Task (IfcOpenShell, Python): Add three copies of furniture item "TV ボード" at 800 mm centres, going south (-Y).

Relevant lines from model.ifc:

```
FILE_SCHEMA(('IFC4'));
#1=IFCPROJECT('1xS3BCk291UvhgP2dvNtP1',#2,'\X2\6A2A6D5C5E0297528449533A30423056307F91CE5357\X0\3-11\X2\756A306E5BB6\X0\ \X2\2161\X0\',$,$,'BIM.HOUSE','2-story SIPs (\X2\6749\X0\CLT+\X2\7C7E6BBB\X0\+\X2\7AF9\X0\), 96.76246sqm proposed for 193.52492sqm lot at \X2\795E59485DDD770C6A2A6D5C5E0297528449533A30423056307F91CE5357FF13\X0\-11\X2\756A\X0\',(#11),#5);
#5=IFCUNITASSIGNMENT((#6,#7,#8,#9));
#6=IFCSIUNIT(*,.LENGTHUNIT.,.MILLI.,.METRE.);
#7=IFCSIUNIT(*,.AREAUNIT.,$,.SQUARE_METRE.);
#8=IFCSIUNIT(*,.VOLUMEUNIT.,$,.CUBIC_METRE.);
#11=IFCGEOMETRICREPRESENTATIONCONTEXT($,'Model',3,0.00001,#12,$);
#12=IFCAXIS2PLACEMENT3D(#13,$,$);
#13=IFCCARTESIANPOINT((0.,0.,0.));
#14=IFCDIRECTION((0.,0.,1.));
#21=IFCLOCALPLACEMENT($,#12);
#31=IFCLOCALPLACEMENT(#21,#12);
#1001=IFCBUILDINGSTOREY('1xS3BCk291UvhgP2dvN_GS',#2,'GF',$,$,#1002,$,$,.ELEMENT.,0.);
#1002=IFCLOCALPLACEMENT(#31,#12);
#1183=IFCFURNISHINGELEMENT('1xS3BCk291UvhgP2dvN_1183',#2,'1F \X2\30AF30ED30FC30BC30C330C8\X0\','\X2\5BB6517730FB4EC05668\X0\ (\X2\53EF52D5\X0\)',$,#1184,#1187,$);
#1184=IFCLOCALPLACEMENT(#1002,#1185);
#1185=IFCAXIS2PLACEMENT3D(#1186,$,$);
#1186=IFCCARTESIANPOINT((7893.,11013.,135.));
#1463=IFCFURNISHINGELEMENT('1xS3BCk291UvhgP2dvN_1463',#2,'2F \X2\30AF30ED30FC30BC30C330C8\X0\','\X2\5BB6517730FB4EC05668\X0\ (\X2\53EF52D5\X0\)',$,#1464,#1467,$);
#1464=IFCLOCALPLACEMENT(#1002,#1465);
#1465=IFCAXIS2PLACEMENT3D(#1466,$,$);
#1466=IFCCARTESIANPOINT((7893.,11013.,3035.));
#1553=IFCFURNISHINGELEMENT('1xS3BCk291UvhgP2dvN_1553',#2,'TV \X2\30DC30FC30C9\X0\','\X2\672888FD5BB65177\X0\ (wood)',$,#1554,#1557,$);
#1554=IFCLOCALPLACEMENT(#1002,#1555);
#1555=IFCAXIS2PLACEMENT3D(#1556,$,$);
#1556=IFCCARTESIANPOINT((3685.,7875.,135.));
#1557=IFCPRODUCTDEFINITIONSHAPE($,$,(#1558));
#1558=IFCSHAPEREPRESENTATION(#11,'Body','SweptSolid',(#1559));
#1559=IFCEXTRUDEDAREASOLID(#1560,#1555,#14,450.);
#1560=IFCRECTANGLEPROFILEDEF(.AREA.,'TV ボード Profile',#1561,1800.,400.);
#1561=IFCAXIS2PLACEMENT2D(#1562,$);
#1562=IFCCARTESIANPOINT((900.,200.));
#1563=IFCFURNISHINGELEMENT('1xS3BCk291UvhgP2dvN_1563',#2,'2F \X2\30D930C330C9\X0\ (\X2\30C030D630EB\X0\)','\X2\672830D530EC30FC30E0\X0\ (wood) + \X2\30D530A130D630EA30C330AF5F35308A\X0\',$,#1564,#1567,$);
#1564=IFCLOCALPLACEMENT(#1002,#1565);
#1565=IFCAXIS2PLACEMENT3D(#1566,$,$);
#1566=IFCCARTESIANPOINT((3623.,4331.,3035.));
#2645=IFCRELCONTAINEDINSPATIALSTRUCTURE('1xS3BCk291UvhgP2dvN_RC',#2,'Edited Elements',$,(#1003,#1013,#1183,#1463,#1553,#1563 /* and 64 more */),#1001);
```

```python
import numpy as np
import ifcopenshell
import ifcopenshell.api.geometry
import ifcopenshell.api.root
import ifcopenshell.util.element
import ifcopenshell.util.placement
import ifcopenshell.util.unit

model = ifcopenshell.open("model.ifc")
unit_scale = ifcopenshell.util.unit.calculate_unit_scale(model)


def reuse_history(source, copy):
    """copy_class also copies each property set's owner history, people and application; keep the originals."""
    for rel in copy.IsDefinedBy:
        if rel.is_a("IfcRelDefinesByProperties") and (history := rel.RelatingPropertyDefinition.OwnerHistory):
            rel.RelatingPropertyDefinition.OwnerHistory = source.OwnerHistory
            ifcopenshell.util.element.remove_deep2(model, history)


source = model.by_guid("1xS3BCk291UvhgP2dvN_1553")
base = ifcopenshell.util.placement.get_local_placement(source.ObjectPlacement)
step = np.array([0.0, -1.0, 0.0]) * 0.8 / unit_scale

for i in range(1, 4):
    copy = ifcopenshell.api.root.copy_class(model, product=source)
    copy.Representation = ifcopenshell.util.element.copy_deep(
        model, source.Representation, exclude=["IfcGeometricRepresentationContext", "IfcRepresentationMap"]
    )
    reuse_history(source, copy)
    matrix = base.copy()
    matrix[:3, 3] += i * step
    print("added at", matrix[:3, 3].round(3) + 0.0)
    ifcopenshell.api.geometry.edit_object_placement(model, product=copy, matrix=matrix, is_si=False)

model.write("model-out.ifc")
```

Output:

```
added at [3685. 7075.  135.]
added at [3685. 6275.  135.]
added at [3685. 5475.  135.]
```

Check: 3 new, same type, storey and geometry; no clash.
